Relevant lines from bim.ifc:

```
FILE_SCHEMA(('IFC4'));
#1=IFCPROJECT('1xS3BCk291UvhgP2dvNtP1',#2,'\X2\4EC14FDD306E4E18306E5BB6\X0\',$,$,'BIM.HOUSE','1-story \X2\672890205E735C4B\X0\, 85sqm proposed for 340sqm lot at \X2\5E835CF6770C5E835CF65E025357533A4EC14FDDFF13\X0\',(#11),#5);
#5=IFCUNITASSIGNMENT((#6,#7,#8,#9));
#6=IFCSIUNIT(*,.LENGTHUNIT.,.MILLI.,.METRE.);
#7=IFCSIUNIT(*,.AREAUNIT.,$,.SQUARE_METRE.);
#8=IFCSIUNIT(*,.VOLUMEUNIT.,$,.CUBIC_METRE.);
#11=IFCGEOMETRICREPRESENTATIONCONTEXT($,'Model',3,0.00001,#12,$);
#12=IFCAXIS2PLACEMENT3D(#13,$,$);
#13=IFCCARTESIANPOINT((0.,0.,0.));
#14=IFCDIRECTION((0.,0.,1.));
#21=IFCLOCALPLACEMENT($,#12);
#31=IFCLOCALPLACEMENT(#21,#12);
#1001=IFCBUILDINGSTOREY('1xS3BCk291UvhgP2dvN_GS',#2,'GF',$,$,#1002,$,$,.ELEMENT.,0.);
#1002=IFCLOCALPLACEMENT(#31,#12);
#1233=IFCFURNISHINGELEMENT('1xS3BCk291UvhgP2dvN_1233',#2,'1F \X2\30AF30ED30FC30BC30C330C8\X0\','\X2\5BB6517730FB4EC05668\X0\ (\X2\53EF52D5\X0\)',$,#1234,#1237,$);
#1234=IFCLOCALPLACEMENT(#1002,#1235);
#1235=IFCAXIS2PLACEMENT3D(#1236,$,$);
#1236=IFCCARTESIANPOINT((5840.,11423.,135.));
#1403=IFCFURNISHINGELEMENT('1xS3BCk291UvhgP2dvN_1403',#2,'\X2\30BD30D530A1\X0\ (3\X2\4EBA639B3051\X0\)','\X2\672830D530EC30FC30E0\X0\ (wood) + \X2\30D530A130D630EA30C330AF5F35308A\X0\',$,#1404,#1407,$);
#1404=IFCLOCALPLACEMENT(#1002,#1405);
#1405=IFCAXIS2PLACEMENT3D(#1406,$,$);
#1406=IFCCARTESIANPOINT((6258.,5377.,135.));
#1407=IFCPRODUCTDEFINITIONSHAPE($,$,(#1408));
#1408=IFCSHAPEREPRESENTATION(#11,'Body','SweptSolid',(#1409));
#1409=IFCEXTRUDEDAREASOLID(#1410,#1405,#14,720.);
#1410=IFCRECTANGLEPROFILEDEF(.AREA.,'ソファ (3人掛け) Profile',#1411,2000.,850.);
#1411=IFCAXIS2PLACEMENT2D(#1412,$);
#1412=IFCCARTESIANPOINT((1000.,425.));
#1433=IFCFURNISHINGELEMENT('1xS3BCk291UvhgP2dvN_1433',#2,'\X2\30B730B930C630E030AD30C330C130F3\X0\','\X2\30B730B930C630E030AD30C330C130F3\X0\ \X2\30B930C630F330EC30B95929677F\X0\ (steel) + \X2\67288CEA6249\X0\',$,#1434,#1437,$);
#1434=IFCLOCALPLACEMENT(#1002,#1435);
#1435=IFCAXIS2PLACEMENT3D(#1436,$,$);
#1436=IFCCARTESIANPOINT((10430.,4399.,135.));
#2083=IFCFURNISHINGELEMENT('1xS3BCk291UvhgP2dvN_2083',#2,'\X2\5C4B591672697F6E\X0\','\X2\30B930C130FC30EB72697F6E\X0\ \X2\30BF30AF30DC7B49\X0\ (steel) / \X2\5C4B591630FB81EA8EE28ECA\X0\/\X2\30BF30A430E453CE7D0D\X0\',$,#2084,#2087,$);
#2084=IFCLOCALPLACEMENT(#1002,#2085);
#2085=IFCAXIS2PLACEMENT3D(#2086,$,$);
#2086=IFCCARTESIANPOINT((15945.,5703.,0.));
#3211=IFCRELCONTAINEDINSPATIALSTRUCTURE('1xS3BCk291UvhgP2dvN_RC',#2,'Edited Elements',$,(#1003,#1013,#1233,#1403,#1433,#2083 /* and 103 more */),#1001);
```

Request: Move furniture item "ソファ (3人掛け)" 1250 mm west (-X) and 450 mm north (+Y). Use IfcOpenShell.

```python
import ifcopenshell
import ifcopenshell.api.geometry
import ifcopenshell.util.placement

model = ifcopenshell.open("bim.ifc")

item = model.by_guid("1xS3BCk291UvhgP2dvN_1403")
matrix = ifcopenshell.util.placement.get_local_placement(item.ObjectPlacement)
matrix[0, 3] -= 1250.0
matrix[1, 3] += 450.0
ifcopenshell.api.geometry.edit_object_placement(model, product=item, matrix=matrix, is_si=False)

print(ifcopenshell.util.placement.get_local_placement(item.ObjectPlacement).round(3) + 0.0)

model.write("bim_rev.ifc")
```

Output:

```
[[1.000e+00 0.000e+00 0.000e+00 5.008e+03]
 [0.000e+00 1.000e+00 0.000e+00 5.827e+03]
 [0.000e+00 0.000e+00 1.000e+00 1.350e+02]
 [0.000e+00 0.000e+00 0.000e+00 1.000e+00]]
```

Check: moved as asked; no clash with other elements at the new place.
